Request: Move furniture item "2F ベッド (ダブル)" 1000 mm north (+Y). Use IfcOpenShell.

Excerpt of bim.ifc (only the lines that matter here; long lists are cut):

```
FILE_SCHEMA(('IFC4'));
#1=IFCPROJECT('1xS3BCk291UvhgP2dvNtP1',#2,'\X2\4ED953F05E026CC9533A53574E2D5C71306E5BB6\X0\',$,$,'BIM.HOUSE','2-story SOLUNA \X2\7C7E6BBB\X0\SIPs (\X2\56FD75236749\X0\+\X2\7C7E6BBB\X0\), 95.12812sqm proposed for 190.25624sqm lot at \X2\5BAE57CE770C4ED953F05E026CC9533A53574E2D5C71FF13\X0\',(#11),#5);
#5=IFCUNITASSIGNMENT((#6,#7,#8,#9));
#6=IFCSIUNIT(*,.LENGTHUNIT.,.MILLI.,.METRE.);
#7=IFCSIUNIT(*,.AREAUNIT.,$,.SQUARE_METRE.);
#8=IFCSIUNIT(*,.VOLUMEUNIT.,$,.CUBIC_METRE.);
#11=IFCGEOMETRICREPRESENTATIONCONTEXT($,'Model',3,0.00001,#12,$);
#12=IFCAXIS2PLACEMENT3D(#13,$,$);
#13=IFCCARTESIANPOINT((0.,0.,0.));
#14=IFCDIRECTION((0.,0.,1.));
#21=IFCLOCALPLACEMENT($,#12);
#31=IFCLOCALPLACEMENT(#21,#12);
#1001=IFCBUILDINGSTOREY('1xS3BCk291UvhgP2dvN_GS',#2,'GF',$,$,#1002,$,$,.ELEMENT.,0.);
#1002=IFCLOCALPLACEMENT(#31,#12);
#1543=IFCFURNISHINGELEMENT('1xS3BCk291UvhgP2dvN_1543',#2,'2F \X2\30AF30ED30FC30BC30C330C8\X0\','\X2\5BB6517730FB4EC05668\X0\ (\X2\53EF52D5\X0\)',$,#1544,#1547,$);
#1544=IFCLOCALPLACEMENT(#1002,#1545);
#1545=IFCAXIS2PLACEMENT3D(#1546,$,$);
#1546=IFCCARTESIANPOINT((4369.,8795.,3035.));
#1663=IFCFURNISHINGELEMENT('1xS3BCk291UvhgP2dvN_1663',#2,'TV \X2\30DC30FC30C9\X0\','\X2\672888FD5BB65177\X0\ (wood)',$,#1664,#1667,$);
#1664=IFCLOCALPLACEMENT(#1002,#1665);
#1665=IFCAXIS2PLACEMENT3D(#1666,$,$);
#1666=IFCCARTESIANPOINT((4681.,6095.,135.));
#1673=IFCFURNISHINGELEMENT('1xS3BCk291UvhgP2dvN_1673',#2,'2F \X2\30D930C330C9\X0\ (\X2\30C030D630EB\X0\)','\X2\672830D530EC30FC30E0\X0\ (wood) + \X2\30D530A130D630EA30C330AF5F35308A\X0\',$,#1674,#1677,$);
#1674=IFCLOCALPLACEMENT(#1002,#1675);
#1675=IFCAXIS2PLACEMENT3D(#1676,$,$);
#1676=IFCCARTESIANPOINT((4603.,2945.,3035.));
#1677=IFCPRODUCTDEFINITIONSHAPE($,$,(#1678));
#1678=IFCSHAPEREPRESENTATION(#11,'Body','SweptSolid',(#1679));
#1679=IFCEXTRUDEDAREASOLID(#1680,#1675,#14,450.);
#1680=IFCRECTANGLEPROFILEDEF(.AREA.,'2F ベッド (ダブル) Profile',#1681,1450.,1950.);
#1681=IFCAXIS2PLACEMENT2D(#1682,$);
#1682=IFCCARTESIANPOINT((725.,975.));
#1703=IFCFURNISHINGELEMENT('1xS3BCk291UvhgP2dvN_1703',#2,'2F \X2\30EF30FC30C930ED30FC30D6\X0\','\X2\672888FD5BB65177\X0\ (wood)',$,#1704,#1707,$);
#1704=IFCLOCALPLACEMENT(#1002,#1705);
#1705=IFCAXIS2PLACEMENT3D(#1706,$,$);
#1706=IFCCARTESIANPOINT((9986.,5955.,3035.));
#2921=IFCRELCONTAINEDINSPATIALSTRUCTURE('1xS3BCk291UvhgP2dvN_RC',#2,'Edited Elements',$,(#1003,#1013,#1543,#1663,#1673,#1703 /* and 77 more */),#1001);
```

```python
import ifcopenshell
import ifcopenshell.api.geometry
import ifcopenshell.util.placement
import ifcopenshell.util.unit

model = ifcopenshell.open("bim.ifc")
unit_scale = ifcopenshell.util.unit.calculate_unit_scale(model)

item = model.by_guid("1xS3BCk291UvhgP2dvN_1673")
matrix = ifcopenshell.util.placement.get_local_placement(item.ObjectPlacement)
matrix[1, 3] += 1 / unit_scale
ifcopenshell.api.geometry.edit_object_placement(model, product=item, matrix=matrix, is_si=False)

print(ifcopenshell.util.placement.get_local_placement(item.ObjectPlacement).round(3) + 0.0)

model.write("bim_v2.ifc")
```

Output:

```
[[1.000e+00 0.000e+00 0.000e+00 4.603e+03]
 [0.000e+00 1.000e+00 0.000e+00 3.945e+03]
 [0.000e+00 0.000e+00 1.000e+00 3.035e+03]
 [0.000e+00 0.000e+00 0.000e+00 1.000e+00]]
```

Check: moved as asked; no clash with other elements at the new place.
